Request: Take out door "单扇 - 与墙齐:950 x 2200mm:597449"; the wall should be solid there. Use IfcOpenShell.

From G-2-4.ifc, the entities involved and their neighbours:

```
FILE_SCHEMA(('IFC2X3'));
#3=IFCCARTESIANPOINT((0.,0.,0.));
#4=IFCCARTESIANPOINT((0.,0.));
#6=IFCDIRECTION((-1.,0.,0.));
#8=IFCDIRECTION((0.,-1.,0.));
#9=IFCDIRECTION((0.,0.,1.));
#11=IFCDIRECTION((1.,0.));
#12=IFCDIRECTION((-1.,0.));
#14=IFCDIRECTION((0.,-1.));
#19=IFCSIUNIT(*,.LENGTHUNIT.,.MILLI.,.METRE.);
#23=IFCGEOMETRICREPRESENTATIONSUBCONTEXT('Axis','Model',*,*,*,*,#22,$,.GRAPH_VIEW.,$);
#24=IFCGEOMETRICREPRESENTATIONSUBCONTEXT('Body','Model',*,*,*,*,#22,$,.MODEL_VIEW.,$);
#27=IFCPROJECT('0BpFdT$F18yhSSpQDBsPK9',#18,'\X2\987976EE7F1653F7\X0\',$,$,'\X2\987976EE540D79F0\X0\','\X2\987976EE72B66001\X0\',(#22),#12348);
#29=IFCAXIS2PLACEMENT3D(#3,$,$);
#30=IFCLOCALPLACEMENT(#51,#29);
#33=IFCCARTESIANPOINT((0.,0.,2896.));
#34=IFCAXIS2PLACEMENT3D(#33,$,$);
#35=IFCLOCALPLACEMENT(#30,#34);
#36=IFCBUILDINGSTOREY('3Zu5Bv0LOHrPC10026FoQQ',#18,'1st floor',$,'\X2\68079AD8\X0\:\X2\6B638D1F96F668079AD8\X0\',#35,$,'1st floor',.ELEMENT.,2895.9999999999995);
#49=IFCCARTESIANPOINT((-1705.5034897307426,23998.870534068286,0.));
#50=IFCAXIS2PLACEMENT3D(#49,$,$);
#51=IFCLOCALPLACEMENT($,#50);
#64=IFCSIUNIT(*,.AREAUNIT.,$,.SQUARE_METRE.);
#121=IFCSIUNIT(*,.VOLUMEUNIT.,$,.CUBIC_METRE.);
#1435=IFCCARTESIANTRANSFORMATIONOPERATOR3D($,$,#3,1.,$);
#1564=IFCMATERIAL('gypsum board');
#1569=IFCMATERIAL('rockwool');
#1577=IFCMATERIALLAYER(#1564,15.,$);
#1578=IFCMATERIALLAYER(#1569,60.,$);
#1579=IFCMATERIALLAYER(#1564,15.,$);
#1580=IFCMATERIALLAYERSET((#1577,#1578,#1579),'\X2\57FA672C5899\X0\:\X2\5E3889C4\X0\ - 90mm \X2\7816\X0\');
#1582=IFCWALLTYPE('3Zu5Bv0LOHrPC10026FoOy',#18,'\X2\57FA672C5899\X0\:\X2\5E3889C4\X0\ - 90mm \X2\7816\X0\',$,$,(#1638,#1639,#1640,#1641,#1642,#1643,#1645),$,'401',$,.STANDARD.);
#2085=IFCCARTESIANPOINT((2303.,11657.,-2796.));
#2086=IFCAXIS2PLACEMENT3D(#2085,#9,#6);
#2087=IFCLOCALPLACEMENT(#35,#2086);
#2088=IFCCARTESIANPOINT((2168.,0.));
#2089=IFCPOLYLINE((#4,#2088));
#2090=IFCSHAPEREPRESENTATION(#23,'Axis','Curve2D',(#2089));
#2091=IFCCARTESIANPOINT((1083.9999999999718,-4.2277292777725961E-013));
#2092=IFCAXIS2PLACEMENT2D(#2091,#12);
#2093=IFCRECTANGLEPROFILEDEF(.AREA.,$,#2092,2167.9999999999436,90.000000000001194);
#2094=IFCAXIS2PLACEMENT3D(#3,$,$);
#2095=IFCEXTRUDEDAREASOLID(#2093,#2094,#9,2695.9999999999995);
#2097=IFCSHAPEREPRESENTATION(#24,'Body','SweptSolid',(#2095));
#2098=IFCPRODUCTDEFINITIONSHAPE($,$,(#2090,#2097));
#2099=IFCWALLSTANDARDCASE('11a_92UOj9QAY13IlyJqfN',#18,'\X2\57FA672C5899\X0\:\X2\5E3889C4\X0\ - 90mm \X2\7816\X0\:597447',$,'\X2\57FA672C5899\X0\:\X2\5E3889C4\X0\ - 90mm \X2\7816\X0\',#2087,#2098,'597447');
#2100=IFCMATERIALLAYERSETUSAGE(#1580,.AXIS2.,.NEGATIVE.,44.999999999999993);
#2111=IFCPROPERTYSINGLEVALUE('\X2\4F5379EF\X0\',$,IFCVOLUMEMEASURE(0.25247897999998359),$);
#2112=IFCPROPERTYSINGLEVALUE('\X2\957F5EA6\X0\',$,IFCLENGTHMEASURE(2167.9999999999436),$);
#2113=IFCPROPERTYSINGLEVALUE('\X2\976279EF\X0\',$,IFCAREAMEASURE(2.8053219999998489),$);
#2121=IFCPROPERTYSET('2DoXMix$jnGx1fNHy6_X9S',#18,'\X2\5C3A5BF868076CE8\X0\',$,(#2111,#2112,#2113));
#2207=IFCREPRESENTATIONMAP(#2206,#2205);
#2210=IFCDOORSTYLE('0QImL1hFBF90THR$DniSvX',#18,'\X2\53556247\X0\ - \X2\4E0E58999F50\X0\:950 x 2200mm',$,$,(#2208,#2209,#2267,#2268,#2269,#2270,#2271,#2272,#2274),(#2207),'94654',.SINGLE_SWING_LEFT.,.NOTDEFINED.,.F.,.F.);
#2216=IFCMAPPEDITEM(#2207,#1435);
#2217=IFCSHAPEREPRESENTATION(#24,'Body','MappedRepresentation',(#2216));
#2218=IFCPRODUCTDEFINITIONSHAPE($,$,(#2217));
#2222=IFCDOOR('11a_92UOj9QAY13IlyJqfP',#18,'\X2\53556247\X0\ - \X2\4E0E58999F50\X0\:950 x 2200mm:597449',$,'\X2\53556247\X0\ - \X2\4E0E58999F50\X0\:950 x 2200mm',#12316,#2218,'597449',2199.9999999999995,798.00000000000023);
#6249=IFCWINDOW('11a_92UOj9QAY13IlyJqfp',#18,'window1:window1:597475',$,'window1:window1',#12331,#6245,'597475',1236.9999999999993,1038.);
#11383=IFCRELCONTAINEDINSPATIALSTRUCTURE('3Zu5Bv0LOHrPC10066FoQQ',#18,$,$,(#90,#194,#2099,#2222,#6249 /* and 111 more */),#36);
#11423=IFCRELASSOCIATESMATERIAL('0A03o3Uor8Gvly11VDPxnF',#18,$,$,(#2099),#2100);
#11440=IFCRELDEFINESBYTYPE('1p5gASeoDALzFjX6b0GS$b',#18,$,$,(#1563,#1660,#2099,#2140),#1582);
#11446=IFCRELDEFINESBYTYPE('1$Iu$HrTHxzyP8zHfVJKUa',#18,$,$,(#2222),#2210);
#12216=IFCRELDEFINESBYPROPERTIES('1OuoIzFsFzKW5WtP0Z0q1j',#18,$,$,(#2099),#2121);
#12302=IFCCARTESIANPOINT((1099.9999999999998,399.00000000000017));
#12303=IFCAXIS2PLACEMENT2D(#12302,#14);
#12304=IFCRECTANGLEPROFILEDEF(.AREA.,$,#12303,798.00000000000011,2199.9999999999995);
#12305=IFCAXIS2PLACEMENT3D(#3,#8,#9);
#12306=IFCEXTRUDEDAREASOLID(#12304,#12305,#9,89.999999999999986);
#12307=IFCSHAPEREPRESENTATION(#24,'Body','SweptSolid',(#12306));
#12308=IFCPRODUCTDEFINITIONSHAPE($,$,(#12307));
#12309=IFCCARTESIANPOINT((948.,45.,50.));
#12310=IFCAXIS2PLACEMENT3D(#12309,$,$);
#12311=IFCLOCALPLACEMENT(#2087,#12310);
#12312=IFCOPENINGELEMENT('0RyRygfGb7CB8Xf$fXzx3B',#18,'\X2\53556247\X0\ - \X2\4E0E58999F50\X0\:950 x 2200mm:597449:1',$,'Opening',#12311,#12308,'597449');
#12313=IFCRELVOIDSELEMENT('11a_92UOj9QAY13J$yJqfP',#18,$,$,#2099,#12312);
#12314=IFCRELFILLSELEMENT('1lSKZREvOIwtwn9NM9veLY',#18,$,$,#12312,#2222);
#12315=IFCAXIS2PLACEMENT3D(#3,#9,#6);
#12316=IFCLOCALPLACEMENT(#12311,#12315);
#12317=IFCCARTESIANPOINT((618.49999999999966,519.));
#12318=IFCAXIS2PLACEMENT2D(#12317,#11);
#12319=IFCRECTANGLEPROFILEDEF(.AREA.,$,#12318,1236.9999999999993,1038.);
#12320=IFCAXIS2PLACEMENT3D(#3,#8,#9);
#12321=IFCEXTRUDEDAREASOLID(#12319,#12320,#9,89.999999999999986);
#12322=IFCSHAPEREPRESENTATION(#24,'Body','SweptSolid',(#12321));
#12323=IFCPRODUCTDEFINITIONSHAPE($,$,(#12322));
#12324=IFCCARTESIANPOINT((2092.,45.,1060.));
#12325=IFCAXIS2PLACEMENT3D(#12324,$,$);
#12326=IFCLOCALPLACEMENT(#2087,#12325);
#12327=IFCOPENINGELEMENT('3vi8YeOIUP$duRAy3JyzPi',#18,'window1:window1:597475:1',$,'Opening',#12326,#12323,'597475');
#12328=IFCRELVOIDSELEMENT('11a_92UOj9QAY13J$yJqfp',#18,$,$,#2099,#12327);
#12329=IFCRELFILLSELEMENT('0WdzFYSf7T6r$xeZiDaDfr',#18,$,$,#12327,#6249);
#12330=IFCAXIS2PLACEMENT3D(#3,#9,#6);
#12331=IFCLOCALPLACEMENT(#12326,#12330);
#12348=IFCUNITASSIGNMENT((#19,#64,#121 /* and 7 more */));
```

```python
import ifcopenshell
import ifcopenshell.api.feature
import ifcopenshell.api.pset
import ifcopenshell.api.root
import ifcopenshell.geom
import ifcopenshell.util.element
import ifcopenshell.util.shape
import ifcopenshell.util.unit

model = ifcopenshell.open("G-2-4.ifc")
area_scale = ifcopenshell.util.unit.calculate_unit_scale(model, "AREAUNIT")
volume_scale = ifcopenshell.util.unit.calculate_unit_scale(model, "VOLUMEUNIT")
settings = ifcopenshell.geom.settings()


def volume(element):
    """Net volume in cubic metres, openings subtracted."""
    shape = ifcopenshell.geom.create_shape(settings, element)
    return ifcopenshell.util.shape.get_volume(shape.geometry)


door = model.by_guid("11a_92UOj9QAY13IlyJqfP")
opening = door.FillsVoids[0].RelatingOpeningElement
wall = opening.VoidsElements[0].RelatingBuildingElement
before = volume(wall)

ifcopenshell.api.root.remove_product(model, product=door)
ifcopenshell.api.feature.remove_feature(model, feature=opening)

after = volume(wall)
thickness = 0.09  # wall thickness in metres

# Update the wall's stored quantities.
pset = model.by_id(ifcopenshell.util.element.get_pset(wall, "尺寸标注", should_inherit=False)["id"])
ifcopenshell.api.pset.edit_pset(model, pset=pset, properties={
    "体积": model.create_entity("IfcVolumeMeasure", after / volume_scale),
    "面积": model.create_entity("IfcAreaMeasure", after / thickness / area_scale),
})

print(f"wall volume {before:.3f} -> {after:.3f} m3")

model.write("G-2-4_rev.ifc")
```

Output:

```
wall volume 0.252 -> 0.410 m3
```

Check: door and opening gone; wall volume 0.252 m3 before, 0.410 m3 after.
